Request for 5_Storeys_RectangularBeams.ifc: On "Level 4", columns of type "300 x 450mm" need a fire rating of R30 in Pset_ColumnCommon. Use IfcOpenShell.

First a look at what the model holds.

```python
import ifcopenshell
import ifcopenshell.util.element

model = ifcopenshell.open("5_Storeys_RectangularBeams.ifc")
print(model.schema)
storey = next(s for s in model.by_type("IfcBuildingStorey") if s.Name == "Level 4")
columns = [e for e in ifcopenshell.util.element.get_decomposition(storey) if e.is_a("IfcColumn")]
seen = {}
for e in columns:
    element_type = ifcopenshell.util.element.get_type(e)
    key = (element_type.Name if element_type != e and element_type else None, ifcopenshell.util.element.get_pset(e, "Pset_ColumnCommon", "FireRating"))
    seen[key] = seen.get(key, 0) + 1
for (name, value), count in sorted(seen.items(), key=str):
    print(count, "x", name, "|", value)
```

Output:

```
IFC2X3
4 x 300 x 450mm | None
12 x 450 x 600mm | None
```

```python
import ifcopenshell
import ifcopenshell.api.pset
import ifcopenshell.util.element

model = ifcopenshell.open("5_Storeys_RectangularBeams.ifc")

storey = next(s for s in model.by_type("IfcBuildingStorey") if s.Name == "Level 4")
columns = [e for e in ifcopenshell.util.element.get_decomposition(storey) if e.is_a("IfcColumn")]

count = 0
for e in columns:
    element_type = ifcopenshell.util.element.get_type(e)
    if element_type in (None, e) or element_type.Name != "300 x 450mm":
        continue
    # add_pset returns the element's existing set when there is one.
    pset = ifcopenshell.api.pset.add_pset(model, product=e, name="Pset_ColumnCommon")
    ifcopenshell.api.pset.edit_pset(model, pset=pset, properties={"FireRating": "R30"})
    count += 1

print(count, "columns updated")

model.write("5_Storeys_RectangularBeams_v2.ifc")
```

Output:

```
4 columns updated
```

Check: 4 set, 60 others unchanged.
